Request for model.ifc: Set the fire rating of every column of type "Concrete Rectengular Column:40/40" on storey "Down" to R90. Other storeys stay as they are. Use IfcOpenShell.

First a look at what the model holds.

```python
import ifcopenshell
import ifcopenshell.util.element

model = ifcopenshell.open("model.ifc")
print(model.schema)
storey = next(s for s in model.by_type("IfcBuildingStorey") if s.Name == "Down")
columns = [e for e in ifcopenshell.util.element.get_decomposition(storey) if e.is_a("IfcColumn")]
seen = {}
for e in columns:
    element_type = ifcopenshell.util.element.get_type(e)
    key = (element_type.Name if element_type != e and element_type else None, ifcopenshell.util.element.get_pset(e, "Pset_ColumnCommon", "FireRating"))
    seen[key] = seen.get(key, 0) + 1
for (name, value), count in sorted(seen.items(), key=str):
    print(count, "x", name, "|", value)
```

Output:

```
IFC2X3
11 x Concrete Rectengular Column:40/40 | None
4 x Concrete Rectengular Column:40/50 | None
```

```python
import ifcopenshell
import ifcopenshell.api.pset
import ifcopenshell.util.element

model = ifcopenshell.open("model.ifc")

storey = next(s for s in model.by_type("IfcBuildingStorey") if s.Name == "Down")
columns = [e for e in ifcopenshell.util.element.get_decomposition(storey) if e.is_a("IfcColumn")]

count = 0
for e in columns:
    element_type = ifcopenshell.util.element.get_type(e)
    if element_type in (None, e) or element_type.Name != "Concrete Rectengular Column:40/40":
        continue
    # add_pset returns the element's existing set when there is one.
    pset = ifcopenshell.api.pset.add_pset(model, product=e, name="Pset_ColumnCommon")
    ifcopenshell.api.pset.edit_pset(model, pset=pset, properties={"FireRating": "R90"})
    count += 1

print(count, "columns updated")

model.write("model_updated.ifc")
```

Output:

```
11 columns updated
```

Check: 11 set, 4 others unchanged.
